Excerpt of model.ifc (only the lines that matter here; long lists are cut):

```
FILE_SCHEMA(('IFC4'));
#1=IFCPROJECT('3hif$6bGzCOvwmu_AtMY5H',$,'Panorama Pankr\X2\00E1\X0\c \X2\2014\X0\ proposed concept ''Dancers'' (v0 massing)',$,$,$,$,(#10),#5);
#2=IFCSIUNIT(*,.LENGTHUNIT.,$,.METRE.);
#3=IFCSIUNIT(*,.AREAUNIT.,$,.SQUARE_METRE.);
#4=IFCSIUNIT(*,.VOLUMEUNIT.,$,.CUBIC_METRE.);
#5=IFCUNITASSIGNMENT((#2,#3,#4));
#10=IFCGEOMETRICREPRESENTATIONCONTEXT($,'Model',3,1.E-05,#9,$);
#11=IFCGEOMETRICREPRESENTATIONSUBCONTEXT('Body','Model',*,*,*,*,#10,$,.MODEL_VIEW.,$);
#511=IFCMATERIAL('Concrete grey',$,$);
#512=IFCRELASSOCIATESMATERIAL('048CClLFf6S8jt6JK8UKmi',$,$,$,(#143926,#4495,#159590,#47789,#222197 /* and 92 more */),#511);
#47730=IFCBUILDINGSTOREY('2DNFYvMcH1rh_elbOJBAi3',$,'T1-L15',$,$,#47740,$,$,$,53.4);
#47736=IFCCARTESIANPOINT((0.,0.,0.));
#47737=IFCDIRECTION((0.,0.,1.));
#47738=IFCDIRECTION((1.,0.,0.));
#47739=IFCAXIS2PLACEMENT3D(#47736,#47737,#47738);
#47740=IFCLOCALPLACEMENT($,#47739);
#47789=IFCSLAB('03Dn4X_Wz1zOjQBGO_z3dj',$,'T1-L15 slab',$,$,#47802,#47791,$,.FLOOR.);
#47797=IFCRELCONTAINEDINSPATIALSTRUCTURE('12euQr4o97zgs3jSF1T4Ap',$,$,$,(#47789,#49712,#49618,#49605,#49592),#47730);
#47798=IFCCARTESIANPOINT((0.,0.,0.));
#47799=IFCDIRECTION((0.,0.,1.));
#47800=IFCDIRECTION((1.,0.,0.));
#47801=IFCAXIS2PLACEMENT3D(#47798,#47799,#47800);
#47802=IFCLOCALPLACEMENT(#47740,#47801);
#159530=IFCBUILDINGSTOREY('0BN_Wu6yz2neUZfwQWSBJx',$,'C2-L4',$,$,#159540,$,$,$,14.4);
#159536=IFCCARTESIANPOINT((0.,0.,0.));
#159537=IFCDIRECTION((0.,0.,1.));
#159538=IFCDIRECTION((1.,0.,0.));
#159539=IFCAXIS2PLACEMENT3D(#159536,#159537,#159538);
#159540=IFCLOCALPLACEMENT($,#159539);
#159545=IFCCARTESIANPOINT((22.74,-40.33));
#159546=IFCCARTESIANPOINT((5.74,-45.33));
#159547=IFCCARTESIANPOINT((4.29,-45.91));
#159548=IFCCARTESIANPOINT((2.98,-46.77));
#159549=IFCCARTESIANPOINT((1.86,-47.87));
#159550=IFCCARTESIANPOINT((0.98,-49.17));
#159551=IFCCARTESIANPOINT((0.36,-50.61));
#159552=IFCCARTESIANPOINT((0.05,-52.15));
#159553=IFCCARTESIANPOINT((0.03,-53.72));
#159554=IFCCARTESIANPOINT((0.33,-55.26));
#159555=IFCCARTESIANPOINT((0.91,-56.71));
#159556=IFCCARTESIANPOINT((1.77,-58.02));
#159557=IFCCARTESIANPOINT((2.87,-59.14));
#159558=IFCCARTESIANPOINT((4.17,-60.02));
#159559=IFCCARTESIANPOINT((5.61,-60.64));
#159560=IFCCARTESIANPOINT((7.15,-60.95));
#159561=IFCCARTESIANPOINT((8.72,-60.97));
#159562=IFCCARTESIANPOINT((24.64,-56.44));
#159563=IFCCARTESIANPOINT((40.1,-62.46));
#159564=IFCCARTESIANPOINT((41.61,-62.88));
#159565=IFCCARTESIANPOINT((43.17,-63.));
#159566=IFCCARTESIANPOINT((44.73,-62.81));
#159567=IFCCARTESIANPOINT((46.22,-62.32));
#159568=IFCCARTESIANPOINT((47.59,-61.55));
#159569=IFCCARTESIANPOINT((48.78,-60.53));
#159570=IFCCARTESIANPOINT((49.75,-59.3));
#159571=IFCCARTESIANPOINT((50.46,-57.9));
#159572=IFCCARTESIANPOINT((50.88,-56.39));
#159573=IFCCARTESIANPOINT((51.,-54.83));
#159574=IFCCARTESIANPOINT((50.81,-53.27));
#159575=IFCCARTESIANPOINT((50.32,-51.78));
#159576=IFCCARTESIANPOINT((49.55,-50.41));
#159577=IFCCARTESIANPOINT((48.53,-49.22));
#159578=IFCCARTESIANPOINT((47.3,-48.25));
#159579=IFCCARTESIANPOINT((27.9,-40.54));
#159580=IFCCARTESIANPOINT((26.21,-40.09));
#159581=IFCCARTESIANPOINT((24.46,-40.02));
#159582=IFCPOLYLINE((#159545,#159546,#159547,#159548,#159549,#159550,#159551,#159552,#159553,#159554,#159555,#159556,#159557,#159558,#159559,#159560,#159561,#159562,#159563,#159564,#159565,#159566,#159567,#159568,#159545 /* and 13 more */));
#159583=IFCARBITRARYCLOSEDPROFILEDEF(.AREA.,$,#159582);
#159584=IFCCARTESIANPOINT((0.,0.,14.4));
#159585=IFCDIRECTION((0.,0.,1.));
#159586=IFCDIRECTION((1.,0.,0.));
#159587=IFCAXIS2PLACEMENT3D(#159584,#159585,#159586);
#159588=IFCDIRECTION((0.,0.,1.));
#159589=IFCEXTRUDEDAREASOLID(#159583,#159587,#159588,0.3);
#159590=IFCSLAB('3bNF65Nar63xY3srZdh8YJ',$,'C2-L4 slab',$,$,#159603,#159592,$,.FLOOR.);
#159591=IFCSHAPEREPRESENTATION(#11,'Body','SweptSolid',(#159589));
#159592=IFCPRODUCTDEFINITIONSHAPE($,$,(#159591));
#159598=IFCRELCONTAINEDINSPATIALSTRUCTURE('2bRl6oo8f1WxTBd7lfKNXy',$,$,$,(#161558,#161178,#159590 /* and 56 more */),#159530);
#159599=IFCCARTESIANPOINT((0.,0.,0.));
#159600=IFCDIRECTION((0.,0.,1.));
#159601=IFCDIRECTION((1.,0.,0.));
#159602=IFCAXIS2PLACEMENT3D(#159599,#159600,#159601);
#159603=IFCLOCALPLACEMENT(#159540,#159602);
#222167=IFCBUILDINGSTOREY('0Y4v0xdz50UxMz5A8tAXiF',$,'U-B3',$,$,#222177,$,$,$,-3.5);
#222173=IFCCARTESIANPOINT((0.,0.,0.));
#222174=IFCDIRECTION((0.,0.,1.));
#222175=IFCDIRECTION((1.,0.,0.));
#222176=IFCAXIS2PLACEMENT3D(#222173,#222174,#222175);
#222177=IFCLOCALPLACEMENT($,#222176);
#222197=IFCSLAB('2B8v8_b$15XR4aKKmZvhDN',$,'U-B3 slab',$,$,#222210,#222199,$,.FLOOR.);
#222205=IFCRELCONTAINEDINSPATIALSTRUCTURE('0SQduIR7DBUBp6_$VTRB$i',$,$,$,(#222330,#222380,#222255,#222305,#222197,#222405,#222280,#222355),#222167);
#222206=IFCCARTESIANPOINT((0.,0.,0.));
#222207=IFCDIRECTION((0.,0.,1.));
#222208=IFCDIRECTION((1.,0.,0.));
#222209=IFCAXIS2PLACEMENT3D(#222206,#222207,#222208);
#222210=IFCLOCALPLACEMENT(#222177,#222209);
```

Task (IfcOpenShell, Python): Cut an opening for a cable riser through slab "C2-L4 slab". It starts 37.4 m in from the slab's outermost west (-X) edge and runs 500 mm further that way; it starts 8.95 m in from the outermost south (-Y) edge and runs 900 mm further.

```python
import numpy as np
import ifcopenshell
import ifcopenshell.api.feature
import ifcopenshell.api.geometry
import ifcopenshell.api.root
import ifcopenshell.geom
import ifcopenshell.util.placement
import ifcopenshell.util.representation
import ifcopenshell.util.shape
import ifcopenshell.util.unit

model = ifcopenshell.open("model.ifc")
unit_scale = ifcopenshell.util.unit.calculate_unit_scale(model)
settings = ifcopenshell.geom.settings()


def volume(element):
    """Net volume in cubic metres, openings subtracted."""
    shape = ifcopenshell.geom.create_shape(settings, element)
    return ifcopenshell.util.shape.get_volume(shape.geometry)


slab = model.by_guid("3bNF65Nar63xY3srZdh8YJ")
before = volume(slab)

# Extent in the slab's own axes, in metres. The edges named are its -X and -Y sides.
slab_shape = ifcopenshell.geom.create_shape(settings, slab)
vertices = ifcopenshell.util.shape.get_vertices(slab_shape.geometry)
x_min, y_min, bottom = vertices.min(axis=0)
top = vertices[:, 2].max()

opening = ifcopenshell.api.root.create_entity(model, ifc_class="IfcOpeningElement", name="Cable riser opening", predefined_type="OPENING")
context = ifcopenshell.util.representation.get_context(model, "Model", "Body", "MODEL_VIEW")
width, depth = 0.5, 0.9
outline = [(0.0, 0.0), (width, 0.0), (width, depth), (0.0, depth), (0.0, 0.0)]
# Overshoot both faces by 50 mm so the cut is clean.
shape = ifcopenshell.api.geometry.add_slab_representation(
    model, context=context, depth=top - bottom + 0.1, polyline=outline
)
ifcopenshell.api.geometry.assign_representation(model, product=opening, representation=shape)

matrix = ifcopenshell.util.placement.get_local_placement(slab.ObjectPlacement)
matrix[:, 3] = matrix @ np.append(np.array([x_min + 37.4, y_min + 8.95, bottom - 0.05]) / unit_scale, 1.0)
ifcopenshell.api.geometry.edit_object_placement(model, product=opening, matrix=matrix, is_si=False)
ifcopenshell.api.feature.add_feature(model, feature=opening, element=slab)

after = volume(slab)

print(f"slab volume {before:.3f} -> {after:.3f} m3")

model.write("model_rev.ifc")
```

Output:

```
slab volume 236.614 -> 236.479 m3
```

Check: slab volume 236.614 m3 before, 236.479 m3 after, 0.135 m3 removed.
